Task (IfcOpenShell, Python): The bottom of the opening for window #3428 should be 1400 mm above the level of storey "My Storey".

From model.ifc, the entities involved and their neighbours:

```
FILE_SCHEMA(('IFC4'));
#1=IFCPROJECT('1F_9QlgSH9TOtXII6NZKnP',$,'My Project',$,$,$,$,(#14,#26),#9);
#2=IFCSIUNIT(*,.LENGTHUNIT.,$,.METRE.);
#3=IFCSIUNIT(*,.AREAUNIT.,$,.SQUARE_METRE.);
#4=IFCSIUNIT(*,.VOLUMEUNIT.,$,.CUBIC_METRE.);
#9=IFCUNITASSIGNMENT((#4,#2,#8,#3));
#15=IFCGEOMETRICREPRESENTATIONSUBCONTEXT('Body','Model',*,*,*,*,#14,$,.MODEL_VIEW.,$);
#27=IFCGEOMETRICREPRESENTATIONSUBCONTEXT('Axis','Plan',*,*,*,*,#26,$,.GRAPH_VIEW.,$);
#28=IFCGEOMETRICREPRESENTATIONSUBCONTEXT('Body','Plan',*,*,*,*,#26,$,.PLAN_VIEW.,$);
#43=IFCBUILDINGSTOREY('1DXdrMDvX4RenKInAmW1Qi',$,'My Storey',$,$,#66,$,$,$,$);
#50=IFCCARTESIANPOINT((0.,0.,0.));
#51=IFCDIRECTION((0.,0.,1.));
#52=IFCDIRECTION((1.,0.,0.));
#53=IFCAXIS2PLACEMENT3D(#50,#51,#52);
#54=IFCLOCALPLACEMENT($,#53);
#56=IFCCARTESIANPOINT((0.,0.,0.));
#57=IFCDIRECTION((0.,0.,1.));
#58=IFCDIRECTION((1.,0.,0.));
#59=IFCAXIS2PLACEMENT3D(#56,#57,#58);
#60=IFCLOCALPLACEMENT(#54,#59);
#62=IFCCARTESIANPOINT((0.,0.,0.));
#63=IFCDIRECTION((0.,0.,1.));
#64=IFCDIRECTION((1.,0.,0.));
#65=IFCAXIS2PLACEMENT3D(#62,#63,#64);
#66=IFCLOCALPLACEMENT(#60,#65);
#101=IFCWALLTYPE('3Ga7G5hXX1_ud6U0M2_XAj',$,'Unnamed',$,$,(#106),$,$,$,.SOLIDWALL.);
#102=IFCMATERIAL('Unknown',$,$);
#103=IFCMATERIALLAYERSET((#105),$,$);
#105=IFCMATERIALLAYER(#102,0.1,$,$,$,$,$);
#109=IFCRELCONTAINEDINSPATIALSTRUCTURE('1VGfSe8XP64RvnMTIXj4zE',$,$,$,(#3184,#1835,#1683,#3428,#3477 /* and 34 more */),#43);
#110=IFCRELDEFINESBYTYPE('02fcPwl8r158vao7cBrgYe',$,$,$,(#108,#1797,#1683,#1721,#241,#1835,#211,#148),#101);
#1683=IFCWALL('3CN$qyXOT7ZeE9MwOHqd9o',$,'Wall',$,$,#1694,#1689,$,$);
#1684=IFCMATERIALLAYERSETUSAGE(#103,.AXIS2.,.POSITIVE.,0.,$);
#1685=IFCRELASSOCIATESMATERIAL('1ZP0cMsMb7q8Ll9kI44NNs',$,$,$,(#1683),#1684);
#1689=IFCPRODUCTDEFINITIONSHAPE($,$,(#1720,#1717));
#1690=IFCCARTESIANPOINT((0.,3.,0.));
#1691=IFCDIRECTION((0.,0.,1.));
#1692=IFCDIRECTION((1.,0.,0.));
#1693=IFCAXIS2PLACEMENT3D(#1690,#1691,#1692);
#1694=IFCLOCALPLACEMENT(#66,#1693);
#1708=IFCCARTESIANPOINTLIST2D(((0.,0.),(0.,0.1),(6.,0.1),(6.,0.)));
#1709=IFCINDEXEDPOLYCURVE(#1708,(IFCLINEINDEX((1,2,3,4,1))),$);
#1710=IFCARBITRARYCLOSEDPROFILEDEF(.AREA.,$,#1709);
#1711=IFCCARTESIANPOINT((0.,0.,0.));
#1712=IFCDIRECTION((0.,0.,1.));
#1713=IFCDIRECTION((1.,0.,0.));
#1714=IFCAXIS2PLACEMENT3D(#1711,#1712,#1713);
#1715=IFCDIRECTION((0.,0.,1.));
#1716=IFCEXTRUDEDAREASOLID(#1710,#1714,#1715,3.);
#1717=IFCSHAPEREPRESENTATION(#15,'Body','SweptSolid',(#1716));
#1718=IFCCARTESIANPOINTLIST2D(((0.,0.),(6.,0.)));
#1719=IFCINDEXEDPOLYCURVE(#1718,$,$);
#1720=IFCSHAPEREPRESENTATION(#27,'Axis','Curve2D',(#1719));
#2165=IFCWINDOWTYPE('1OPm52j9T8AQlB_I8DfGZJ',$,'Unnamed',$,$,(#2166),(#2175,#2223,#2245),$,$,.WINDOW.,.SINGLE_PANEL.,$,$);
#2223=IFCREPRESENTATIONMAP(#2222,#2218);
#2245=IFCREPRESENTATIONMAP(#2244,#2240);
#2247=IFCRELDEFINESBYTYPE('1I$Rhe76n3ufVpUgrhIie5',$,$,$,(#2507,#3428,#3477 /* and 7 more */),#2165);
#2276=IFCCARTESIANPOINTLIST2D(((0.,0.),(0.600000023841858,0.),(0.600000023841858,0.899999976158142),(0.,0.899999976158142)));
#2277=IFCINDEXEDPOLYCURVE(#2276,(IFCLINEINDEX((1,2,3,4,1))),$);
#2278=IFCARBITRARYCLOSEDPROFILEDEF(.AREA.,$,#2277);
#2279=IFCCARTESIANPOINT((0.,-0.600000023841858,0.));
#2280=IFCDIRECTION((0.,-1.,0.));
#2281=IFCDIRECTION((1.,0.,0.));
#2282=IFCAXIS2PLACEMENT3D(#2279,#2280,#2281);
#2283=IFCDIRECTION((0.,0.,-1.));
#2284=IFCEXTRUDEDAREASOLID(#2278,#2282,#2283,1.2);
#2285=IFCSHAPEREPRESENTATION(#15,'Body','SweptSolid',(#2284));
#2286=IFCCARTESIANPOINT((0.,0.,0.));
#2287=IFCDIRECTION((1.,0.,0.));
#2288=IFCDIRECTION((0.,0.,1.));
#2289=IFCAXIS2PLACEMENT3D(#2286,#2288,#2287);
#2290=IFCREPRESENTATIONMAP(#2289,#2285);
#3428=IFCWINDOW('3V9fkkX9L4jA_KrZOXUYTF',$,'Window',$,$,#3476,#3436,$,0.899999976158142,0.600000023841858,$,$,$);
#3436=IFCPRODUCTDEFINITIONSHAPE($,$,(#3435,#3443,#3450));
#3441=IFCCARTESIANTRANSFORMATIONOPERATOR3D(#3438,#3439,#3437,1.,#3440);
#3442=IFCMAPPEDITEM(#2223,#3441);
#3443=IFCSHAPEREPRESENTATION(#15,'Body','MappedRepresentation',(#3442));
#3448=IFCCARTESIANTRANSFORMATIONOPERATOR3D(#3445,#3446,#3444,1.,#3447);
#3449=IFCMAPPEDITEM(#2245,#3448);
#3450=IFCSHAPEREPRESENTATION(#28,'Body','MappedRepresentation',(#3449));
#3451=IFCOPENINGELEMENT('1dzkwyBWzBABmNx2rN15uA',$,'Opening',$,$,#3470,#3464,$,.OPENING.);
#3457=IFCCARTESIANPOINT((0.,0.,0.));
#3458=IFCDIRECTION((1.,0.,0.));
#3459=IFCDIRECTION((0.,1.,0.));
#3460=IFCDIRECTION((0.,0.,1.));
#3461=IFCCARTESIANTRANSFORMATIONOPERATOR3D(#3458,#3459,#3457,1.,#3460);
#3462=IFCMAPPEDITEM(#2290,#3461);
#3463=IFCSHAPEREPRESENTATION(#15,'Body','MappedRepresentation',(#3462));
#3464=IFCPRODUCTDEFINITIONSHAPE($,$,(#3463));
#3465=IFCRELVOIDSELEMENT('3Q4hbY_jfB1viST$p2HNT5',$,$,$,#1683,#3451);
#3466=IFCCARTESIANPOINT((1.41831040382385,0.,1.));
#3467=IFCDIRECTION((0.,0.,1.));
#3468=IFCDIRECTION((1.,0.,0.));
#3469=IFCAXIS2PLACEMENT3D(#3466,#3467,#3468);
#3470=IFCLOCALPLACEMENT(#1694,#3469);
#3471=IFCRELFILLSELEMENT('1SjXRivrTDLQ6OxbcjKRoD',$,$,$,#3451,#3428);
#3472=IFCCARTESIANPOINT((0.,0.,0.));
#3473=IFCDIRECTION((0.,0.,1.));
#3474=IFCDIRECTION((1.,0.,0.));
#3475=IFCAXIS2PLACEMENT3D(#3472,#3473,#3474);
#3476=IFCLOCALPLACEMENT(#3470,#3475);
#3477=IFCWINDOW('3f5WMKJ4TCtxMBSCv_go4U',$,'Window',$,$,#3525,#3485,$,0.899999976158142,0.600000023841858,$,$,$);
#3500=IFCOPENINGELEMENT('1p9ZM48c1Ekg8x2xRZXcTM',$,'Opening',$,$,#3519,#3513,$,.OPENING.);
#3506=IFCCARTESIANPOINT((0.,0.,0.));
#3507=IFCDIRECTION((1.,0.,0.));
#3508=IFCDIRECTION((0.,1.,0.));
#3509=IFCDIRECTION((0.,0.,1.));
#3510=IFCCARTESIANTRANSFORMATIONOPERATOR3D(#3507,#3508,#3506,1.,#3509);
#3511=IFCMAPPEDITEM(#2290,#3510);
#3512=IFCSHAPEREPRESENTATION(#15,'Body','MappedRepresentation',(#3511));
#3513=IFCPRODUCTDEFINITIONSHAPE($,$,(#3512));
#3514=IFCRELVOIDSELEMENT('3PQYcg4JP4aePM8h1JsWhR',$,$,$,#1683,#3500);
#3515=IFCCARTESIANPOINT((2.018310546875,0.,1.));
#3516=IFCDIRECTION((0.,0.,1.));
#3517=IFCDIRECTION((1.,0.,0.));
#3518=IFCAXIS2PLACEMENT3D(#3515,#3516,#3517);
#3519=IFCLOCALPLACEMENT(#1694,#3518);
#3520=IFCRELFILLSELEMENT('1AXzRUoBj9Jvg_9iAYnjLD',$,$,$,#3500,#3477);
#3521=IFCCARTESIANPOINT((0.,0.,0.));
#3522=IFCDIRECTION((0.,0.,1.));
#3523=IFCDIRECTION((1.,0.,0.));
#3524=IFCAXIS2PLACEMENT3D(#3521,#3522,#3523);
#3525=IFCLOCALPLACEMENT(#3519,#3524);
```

```python
import numpy as np
import ifcopenshell
import ifcopenshell.api.geometry
import ifcopenshell.geom
import ifcopenshell.util.element
import ifcopenshell.util.placement
import ifcopenshell.util.shape
import ifcopenshell.util.unit

model = ifcopenshell.open("model.ifc")
unit_scale = ifcopenshell.util.unit.calculate_unit_scale(model)

window = model.by_guid("3V9fkkX9L4jA_KrZOXUYTF")
opening = window.FillsVoids[0].RelatingOpeningElement
storey = ifcopenshell.util.element.get_container(window, ifc_class="IfcBuildingStorey")
level = ifcopenshell.util.placement.get_local_placement(storey.ObjectPlacement)[2, 3]

# The opening's origin need not be at the sill, so measure its lowest point.
shape = ifcopenshell.geom.create_shape(ifcopenshell.geom.settings(), opening)
bottom = ifcopenshell.util.shape.get_shape_bottom_elevation(shape, shape.geometry) / unit_scale
dz = level + 1.4 / unit_scale - bottom

shift = np.array([0.0, 0.0, dz])
# The window is placed relative to its opening, so it follows when the opening moves.
matrix = ifcopenshell.util.placement.get_local_placement(opening.ObjectPlacement)
matrix[:3, 3] += shift
ifcopenshell.api.geometry.edit_object_placement(
    model, product=opening, matrix=matrix, is_si=False, should_transform_children=True
)

print(f"moved by {dz * unit_scale:+.3f} m")

model.write("model_rev.ifc")
```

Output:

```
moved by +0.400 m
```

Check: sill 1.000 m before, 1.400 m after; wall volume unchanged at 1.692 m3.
